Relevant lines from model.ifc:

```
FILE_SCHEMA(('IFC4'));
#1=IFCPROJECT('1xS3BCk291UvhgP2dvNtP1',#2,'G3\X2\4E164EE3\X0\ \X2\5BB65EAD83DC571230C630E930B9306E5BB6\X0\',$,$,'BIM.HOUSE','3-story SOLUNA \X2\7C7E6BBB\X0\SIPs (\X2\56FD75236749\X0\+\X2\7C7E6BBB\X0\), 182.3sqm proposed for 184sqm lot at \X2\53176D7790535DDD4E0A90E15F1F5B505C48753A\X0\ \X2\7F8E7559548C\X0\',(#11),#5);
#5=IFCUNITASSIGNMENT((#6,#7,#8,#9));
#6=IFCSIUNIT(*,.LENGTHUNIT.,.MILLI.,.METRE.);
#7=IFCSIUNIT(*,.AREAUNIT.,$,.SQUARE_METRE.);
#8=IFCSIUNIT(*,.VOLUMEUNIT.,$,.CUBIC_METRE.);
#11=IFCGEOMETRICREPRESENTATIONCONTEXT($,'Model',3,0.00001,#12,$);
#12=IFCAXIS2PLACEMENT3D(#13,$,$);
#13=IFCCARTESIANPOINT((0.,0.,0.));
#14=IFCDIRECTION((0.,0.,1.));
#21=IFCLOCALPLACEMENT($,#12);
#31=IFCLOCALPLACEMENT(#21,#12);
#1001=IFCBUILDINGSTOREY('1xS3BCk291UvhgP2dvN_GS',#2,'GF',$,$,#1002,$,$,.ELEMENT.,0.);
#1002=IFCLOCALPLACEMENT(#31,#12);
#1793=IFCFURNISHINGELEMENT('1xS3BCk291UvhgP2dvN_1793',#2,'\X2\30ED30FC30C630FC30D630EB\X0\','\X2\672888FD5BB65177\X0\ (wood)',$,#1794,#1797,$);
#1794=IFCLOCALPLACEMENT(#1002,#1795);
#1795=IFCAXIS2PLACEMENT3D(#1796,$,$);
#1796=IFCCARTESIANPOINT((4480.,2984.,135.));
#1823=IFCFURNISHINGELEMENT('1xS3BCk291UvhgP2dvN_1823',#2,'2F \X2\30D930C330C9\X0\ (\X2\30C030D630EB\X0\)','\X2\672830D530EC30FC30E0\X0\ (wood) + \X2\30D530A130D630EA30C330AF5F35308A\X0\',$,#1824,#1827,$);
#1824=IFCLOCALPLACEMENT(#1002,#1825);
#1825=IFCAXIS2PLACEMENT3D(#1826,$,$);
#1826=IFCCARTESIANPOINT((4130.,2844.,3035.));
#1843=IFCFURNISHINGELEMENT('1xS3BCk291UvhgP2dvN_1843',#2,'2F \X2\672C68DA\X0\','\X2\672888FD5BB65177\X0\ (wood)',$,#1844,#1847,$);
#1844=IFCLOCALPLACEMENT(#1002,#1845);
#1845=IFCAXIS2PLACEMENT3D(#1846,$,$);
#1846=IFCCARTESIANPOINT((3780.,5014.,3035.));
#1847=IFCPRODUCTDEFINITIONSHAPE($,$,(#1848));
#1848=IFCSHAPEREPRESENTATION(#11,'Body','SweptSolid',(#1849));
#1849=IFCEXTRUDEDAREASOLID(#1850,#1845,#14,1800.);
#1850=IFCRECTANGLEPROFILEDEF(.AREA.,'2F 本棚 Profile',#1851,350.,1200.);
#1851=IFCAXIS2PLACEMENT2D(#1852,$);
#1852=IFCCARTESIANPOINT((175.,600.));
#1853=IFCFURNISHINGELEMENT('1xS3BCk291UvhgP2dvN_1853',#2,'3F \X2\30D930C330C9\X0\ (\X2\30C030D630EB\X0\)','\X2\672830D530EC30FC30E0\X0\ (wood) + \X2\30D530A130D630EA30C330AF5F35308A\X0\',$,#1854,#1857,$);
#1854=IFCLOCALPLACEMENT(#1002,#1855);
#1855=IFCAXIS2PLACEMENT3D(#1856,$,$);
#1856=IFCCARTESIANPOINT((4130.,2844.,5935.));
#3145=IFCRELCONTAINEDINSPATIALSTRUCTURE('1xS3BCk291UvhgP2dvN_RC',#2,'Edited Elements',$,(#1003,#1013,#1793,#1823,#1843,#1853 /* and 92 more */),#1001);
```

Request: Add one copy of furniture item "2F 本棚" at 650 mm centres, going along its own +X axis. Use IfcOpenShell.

```python
import ifcopenshell
import ifcopenshell.api.geometry
import ifcopenshell.api.root
import ifcopenshell.util.element
import ifcopenshell.util.placement

model = ifcopenshell.open("model.ifc")


def reuse_history(source, copy):
    """copy_class also copies each property set's owner history, people and application; keep the originals."""
    for rel in copy.IsDefinedBy:
        if rel.is_a("IfcRelDefinesByProperties") and (history := rel.RelatingPropertyDefinition.OwnerHistory):
            rel.RelatingPropertyDefinition.OwnerHistory = source.OwnerHistory
            ifcopenshell.util.element.remove_deep2(model, history)


source = model.by_guid("1xS3BCk291UvhgP2dvN_1843")
base = ifcopenshell.util.placement.get_local_placement(source.ObjectPlacement)
step = base[:3, 0] * 650.0

for i in range(1, 2):
    copy = ifcopenshell.api.root.copy_class(model, product=source)
    copy.Representation = ifcopenshell.util.element.copy_deep(
        model, source.Representation, exclude=["IfcGeometricRepresentationContext", "IfcRepresentationMap"]
    )
    reuse_history(source, copy)
    matrix = base.copy()
    matrix[:3, 3] += i * step
    print("added at", matrix[:3, 3].round(3) + 0.0)
    ifcopenshell.api.geometry.edit_object_placement(model, product=copy, matrix=matrix, is_si=False)

model.write("model_updated.ifc")
```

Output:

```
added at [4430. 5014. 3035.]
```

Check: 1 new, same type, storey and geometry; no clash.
